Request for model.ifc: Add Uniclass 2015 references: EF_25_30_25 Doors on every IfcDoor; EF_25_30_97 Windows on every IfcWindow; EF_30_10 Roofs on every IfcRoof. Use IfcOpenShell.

First a look at what the model holds.

```python
import ifcopenshell

model = ifcopenshell.open("model.ifc")
print(model.schema)
print("classifications:", [c.Name for c in model.by_type("IfcClassification")])
for ifc_class in ("IfcDoor", "IfcRoof", "IfcStair", "IfcWall", "IfcWindow"):
    print(ifc_class, len(model.by_type(ifc_class)))
```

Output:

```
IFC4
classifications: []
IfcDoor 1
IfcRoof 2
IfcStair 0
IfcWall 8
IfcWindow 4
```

```python
import ifcopenshell
import ifcopenshell.api.classification

model = ifcopenshell.open("model.ifc")

system = ifcopenshell.api.classification.add_classification(model, classification="Uniclass 2015")

codes = {
    "IfcDoor": ("EF_25_30_25", "Doors"),
    "IfcWindow": ("EF_25_30_97", "Windows"),
    "IfcRoof": ("EF_30_10", "Roofs"),
}
for ifc_class, (code, name) in codes.items():
    products = model.by_type(ifc_class)
    ifcopenshell.api.classification.add_reference(
        model, products=products, classification=system, identification=code, name=name
    )
    print(code, len(products))

model.write("model-out.ifc")
```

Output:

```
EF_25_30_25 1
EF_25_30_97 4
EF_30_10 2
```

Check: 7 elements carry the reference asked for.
